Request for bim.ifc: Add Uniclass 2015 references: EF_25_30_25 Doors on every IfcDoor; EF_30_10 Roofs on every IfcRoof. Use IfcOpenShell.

First a look at what the model holds.

```python
import ifcopenshell

model = ifcopenshell.open("bim.ifc")
print(model.schema)
print("classifications:", [c.Name for c in model.by_type("IfcClassification")])
for ifc_class in ("IfcDoor", "IfcRoof", "IfcStair", "IfcWall", "IfcWindow"):
    print(ifc_class, len(model.by_type(ifc_class)))
```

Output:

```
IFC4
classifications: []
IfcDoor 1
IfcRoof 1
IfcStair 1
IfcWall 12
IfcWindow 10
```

```python
import ifcopenshell
import ifcopenshell.api.classification

model = ifcopenshell.open("bim.ifc")

system = ifcopenshell.api.classification.add_classification(model, classification="Uniclass 2015")

codes = {
    "IfcDoor": ("EF_25_30_25", "Doors"),
    "IfcRoof": ("EF_30_10", "Roofs"),
}
for ifc_class, (code, name) in codes.items():
    products = model.by_type(ifc_class)
    ifcopenshell.api.classification.add_reference(
        model, products=products, classification=system, identification=code, name=name
    )
    print(code, len(products))

model.write("bim_v2.ifc")
```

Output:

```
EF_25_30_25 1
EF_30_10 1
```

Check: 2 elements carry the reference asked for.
